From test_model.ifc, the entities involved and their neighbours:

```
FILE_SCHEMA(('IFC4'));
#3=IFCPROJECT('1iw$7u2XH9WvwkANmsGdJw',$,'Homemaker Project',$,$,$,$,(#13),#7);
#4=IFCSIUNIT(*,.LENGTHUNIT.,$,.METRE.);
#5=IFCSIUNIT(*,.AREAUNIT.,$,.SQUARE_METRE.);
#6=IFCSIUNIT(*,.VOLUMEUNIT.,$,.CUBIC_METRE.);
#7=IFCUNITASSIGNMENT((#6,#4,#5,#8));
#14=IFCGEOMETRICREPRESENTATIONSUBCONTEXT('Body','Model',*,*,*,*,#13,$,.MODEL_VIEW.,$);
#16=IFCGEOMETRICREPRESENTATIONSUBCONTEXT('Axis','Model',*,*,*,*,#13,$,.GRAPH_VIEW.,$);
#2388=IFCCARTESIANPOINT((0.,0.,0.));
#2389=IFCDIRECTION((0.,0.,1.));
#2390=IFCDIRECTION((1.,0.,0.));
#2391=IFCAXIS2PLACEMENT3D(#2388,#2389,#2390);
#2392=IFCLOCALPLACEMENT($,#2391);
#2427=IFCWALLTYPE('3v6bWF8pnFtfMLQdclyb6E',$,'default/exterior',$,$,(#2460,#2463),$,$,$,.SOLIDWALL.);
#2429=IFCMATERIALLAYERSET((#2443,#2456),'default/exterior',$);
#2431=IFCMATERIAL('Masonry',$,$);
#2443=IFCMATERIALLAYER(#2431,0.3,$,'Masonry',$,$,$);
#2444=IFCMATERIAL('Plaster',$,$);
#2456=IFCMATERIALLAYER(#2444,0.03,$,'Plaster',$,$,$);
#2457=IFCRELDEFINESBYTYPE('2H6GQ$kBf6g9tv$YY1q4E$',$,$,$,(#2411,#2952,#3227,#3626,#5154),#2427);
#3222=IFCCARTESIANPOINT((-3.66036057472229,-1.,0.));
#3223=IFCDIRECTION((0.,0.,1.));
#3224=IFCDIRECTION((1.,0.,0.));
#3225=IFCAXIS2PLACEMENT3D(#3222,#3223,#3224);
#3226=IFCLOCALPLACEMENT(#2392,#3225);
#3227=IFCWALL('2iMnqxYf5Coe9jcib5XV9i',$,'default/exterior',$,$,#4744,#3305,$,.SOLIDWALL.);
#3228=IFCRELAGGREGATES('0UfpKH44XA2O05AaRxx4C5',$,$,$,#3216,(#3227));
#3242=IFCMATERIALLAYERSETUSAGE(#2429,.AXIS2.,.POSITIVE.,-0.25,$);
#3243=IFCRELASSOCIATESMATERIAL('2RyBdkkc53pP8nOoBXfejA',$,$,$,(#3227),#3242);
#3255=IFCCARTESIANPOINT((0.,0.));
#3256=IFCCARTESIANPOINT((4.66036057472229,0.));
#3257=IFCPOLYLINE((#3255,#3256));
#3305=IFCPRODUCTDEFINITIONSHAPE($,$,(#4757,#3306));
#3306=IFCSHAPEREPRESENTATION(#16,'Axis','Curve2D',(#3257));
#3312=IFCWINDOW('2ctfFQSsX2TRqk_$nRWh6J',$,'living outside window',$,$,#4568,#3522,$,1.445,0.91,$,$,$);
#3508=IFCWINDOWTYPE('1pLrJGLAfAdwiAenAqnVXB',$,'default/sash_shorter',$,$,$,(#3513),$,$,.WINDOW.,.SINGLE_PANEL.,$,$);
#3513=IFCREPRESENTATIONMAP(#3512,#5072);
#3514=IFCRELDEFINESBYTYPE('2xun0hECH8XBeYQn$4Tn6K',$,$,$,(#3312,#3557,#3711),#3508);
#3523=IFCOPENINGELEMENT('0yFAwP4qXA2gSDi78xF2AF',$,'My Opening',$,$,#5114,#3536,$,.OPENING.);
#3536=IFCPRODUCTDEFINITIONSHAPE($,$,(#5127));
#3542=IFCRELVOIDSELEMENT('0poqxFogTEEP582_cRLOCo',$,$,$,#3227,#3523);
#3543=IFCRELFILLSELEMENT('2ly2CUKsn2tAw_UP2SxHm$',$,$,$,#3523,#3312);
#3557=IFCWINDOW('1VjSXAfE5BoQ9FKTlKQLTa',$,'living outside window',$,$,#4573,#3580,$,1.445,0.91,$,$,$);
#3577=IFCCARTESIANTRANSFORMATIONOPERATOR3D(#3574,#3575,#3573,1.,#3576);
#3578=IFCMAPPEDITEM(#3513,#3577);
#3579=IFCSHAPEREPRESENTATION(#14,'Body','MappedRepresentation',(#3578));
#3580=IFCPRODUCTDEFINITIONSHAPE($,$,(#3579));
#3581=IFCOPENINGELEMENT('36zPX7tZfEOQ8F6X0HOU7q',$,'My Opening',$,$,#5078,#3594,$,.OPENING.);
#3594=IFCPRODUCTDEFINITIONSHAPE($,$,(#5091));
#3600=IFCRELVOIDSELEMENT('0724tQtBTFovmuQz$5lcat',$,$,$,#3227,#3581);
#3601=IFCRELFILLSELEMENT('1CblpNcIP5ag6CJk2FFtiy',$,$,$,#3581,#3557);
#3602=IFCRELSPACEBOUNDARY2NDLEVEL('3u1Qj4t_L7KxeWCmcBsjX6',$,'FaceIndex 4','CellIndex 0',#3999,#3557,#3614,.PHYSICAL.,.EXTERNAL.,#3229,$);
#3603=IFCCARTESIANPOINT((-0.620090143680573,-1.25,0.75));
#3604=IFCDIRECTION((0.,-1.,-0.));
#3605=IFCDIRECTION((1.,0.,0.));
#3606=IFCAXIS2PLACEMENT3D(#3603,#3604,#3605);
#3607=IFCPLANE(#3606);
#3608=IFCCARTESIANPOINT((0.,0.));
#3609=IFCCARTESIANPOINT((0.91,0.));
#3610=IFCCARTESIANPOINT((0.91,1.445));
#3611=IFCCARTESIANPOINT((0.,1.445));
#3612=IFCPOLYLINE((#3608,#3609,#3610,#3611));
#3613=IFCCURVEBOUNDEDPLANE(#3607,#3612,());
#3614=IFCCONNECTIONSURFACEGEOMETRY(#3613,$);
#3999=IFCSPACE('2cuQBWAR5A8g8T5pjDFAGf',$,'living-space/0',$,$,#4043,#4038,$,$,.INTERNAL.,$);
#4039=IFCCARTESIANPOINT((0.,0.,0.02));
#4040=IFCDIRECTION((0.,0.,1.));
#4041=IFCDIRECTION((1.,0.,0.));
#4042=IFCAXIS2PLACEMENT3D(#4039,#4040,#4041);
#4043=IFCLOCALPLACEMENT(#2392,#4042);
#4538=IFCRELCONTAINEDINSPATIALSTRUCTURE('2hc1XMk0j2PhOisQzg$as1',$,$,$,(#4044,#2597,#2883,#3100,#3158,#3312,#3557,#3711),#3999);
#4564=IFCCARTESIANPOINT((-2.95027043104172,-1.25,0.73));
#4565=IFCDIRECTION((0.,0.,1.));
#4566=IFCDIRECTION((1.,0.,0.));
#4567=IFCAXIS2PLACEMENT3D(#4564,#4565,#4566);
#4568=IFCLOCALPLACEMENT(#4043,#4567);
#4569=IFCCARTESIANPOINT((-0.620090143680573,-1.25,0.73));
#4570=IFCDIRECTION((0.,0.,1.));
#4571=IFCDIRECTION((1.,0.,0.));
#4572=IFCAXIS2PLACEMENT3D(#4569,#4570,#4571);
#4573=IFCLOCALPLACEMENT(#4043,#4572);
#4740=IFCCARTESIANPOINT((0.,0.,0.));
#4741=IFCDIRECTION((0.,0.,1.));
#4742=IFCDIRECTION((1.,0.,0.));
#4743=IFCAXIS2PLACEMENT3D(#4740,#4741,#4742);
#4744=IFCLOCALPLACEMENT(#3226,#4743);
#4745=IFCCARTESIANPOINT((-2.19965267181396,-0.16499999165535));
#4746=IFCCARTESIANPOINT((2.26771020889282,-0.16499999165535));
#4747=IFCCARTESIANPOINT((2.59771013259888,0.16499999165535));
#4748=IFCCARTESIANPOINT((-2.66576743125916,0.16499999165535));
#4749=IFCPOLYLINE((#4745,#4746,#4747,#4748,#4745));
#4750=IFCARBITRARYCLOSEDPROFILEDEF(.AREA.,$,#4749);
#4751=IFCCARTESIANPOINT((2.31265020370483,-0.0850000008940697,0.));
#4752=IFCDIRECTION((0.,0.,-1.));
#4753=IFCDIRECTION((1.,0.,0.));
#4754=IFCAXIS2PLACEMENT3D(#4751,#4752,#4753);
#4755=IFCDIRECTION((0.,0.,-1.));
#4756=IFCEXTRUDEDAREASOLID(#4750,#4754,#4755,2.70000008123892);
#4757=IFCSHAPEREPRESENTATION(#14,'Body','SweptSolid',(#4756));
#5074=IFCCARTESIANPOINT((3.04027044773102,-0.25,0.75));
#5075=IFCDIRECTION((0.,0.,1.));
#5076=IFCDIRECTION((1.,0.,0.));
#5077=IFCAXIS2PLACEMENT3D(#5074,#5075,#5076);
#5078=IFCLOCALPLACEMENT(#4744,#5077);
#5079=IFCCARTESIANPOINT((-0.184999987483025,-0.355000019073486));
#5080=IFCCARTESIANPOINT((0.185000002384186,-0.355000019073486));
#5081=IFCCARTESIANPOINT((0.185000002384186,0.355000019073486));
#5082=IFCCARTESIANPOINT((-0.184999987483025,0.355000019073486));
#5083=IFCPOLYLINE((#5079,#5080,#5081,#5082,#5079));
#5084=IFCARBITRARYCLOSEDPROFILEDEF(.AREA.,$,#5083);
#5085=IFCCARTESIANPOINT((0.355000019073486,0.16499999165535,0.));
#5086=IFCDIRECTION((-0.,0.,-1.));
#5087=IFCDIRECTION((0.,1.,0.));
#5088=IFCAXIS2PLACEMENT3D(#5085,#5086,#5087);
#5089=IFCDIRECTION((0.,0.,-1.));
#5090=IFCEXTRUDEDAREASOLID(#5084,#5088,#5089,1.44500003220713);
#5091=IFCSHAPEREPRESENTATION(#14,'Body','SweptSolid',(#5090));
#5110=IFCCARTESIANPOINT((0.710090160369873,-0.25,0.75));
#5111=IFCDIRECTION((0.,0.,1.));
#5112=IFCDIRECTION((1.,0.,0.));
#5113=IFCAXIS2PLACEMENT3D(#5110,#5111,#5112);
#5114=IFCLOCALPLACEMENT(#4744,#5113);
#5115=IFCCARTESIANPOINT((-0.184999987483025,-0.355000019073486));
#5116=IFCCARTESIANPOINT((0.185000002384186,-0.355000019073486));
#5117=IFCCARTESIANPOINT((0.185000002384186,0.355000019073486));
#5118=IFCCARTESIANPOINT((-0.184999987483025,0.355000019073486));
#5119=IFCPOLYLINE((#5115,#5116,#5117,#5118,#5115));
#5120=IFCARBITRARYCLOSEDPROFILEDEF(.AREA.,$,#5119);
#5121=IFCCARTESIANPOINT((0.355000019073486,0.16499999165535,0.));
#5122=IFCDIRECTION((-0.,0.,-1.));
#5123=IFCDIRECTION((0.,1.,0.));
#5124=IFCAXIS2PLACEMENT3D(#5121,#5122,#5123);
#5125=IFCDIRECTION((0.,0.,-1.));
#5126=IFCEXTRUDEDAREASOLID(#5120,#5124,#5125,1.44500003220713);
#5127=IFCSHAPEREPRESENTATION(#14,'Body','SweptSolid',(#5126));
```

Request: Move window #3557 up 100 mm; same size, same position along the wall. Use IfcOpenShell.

```python
import numpy as np
import ifcopenshell
import ifcopenshell.api.geometry
import ifcopenshell.util.placement
import ifcopenshell.util.unit

model = ifcopenshell.open("test_model.ifc")
unit_scale = ifcopenshell.util.unit.calculate_unit_scale(model)

window = model.by_id(3557)
opening = window.FillsVoids[0].RelatingOpeningElement
dz = 0.1 / unit_scale

shift = np.array([0.0, 0.0, dz])
# The window is not placed relative to its opening, so move both.
for product in (opening, window):
    matrix = ifcopenshell.util.placement.get_local_placement(product.ObjectPlacement)
    matrix[:3, 3] += shift
    ifcopenshell.api.geometry.edit_object_placement(model, product=product, matrix=matrix, is_si=False)

# Space boundary surfaces are stored in each space's coordinates; move them too.
for rel in window.ProvidesBoundaries:
    if not rel.ConnectionGeometry:
        continue
    surface = rel.ConnectionGeometry.SurfaceOnRelatingElement.BasisSurface
    space_matrix = ifcopenshell.util.placement.get_local_placement(rel.RelatingSpace.ObjectPlacement)
    point = np.array(surface.Position.Location.Coordinates) + space_matrix[:3, :3].T @ shift
    surface.Position = model.createIfcAxis2Placement3D(
        model.createIfcCartesianPoint(point.tolist()), surface.Position.Axis, surface.Position.RefDirection
    )

print(f"moved by {dz * unit_scale:+.3f} m")

model.write("test_model_updated.ifc")
```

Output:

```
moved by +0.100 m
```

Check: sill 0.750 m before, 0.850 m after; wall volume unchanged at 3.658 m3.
